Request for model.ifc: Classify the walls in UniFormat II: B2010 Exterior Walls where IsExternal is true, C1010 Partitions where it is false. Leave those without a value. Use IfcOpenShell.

First a look at what the model holds.

```python
import ifcopenshell
import ifcopenshell.util.element

model = ifcopenshell.open("model.ifc")
print(model.schema)
print("classifications:", [c.Name for c in model.by_type("IfcClassification")])
values = [ifcopenshell.util.element.get_pset(e, "Pset_WallCommon", "IsExternal") for e in model.by_type("IfcWall")]
for value in (True, False, None):
    print("IsExternal", value, values.count(value))
```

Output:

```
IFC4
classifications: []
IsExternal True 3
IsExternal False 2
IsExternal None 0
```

```python
import ifcopenshell
import ifcopenshell.api.classification
import ifcopenshell.util.element

model = ifcopenshell.open("model.ifc")

system = ifcopenshell.api.classification.add_classification(model, classification="UniFormat II")

walls = model.by_type("IfcWall")
external = {e: ifcopenshell.util.element.get_pset(e, "Pset_WallCommon", "IsExternal") for e in walls}
for flag, code, name in ((True, "B2010", "Exterior Walls"), (False, "C1010", "Partitions")):
    products = [e for e in walls if external[e] is flag]
    ifcopenshell.api.classification.add_reference(
        model, products=products, classification=system, identification=code, name=name
    )
    print(code, len(products))

model.write("model_edited.ifc")
```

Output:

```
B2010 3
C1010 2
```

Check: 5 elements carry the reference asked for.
